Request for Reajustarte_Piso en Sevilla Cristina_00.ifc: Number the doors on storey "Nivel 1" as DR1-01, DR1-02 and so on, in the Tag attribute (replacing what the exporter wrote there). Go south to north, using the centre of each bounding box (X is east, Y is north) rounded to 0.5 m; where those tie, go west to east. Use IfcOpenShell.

First a look at what the model holds.

```python
import ifcopenshell
import ifcopenshell.util.element
import ifcopenshell.util.placement

model = ifcopenshell.open("Reajustarte_Piso en Sevilla Cristina_00.ifc")
print(model.schema)
storey = next(s for s in model.by_type("IfcBuildingStorey") if s.Name == "Nivel 1")
doors = [e for e in ifcopenshell.util.element.get_decomposition(storey) if e.is_a("IfcDoor")]
for e in sorted(doors, key=lambda e: e.id()):
    origin = ifcopenshell.util.placement.get_local_placement(e.ObjectPlacement)[:3, 3]
    print(e.id(), e.Tag, e.Name, origin.round(2) + 0.0, sep=" | ")
```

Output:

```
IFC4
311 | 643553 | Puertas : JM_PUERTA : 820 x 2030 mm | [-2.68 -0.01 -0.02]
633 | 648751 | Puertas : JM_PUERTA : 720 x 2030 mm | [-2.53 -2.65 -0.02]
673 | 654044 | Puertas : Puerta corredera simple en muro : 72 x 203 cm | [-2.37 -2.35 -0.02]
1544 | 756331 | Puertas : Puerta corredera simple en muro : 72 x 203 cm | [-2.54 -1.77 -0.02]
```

```python
import ifcopenshell
import ifcopenshell.geom
import ifcopenshell.util.element
import ifcopenshell.util.shape

model = ifcopenshell.open("Reajustarte_Piso en Sevilla Cristina_00.ifc")
settings = ifcopenshell.geom.settings()
settings.set("use-world-coords", True)


def centre(element):
    shape = ifcopenshell.geom.create_shape(settings, element)
    return ifcopenshell.util.shape.get_bbox_centroid(shape.geometry)


storey = next(s for s in model.by_type("IfcBuildingStorey") if s.Name == "Nivel 1")
doors = [e for e in ifcopenshell.util.element.get_decomposition(storey) if e.is_a("IfcDoor")]

# Insertion points can sit at a corner or the storey origin, so sort by the geometry (in metres).
centres = {e: centre(e) for e in doors}
doors.sort(key=lambda e: (round(centres[e][1] / 0.5), centres[e][0]))

for i, e in enumerate(doors, start=1):
    number = f"DR1-{i:02d}"
    e.Tag = number
    print(e.id(), number)

model.write("Reajustarte_Piso en Sevilla Cristina_00-out.ifc")
```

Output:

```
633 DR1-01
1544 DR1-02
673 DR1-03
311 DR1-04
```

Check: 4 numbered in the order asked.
